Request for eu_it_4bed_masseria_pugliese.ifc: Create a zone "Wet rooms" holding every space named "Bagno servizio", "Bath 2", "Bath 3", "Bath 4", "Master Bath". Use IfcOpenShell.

First a look at what the model holds.

```python
import ifcopenshell

model = ifcopenshell.open("eu_it_4bed_masseria_pugliese.ifc")
print(model.schema)
seen = {}
for space in model.by_type("IfcSpace"):
    seen[space.LongName] = seen.get(space.LongName, 0) + 1
for name, count in sorted(seen.items(), key=str):
    print(count, "x", name)
print("zones:", [z.Name for z in model.by_type("IfcZone")][:20])
```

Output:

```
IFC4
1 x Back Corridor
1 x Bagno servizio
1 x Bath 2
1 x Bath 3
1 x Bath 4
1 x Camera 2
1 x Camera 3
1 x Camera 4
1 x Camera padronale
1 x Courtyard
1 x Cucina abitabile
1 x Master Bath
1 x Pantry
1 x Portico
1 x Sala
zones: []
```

```python
import ifcopenshell
import ifcopenshell.api.group
import ifcopenshell.api.root

model = ifcopenshell.open("eu_it_4bed_masseria_pugliese.ifc")

names = {"Bagno servizio", "Bath 2", "Bath 3", "Bath 4", "Master Bath"}
spaces = [s for s in model.by_type("IfcSpace") if s.LongName in names]

zone = ifcopenshell.api.root.create_entity(model, ifc_class="IfcZone", name="Wet rooms")
ifcopenshell.api.group.assign_group(model, products=spaces, group=zone)
print(len(spaces), "spaces in", zone.Name)

model.write("eu_it_4bed_masseria_pugliese_updated.ifc")
```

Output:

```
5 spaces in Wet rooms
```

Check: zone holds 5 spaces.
